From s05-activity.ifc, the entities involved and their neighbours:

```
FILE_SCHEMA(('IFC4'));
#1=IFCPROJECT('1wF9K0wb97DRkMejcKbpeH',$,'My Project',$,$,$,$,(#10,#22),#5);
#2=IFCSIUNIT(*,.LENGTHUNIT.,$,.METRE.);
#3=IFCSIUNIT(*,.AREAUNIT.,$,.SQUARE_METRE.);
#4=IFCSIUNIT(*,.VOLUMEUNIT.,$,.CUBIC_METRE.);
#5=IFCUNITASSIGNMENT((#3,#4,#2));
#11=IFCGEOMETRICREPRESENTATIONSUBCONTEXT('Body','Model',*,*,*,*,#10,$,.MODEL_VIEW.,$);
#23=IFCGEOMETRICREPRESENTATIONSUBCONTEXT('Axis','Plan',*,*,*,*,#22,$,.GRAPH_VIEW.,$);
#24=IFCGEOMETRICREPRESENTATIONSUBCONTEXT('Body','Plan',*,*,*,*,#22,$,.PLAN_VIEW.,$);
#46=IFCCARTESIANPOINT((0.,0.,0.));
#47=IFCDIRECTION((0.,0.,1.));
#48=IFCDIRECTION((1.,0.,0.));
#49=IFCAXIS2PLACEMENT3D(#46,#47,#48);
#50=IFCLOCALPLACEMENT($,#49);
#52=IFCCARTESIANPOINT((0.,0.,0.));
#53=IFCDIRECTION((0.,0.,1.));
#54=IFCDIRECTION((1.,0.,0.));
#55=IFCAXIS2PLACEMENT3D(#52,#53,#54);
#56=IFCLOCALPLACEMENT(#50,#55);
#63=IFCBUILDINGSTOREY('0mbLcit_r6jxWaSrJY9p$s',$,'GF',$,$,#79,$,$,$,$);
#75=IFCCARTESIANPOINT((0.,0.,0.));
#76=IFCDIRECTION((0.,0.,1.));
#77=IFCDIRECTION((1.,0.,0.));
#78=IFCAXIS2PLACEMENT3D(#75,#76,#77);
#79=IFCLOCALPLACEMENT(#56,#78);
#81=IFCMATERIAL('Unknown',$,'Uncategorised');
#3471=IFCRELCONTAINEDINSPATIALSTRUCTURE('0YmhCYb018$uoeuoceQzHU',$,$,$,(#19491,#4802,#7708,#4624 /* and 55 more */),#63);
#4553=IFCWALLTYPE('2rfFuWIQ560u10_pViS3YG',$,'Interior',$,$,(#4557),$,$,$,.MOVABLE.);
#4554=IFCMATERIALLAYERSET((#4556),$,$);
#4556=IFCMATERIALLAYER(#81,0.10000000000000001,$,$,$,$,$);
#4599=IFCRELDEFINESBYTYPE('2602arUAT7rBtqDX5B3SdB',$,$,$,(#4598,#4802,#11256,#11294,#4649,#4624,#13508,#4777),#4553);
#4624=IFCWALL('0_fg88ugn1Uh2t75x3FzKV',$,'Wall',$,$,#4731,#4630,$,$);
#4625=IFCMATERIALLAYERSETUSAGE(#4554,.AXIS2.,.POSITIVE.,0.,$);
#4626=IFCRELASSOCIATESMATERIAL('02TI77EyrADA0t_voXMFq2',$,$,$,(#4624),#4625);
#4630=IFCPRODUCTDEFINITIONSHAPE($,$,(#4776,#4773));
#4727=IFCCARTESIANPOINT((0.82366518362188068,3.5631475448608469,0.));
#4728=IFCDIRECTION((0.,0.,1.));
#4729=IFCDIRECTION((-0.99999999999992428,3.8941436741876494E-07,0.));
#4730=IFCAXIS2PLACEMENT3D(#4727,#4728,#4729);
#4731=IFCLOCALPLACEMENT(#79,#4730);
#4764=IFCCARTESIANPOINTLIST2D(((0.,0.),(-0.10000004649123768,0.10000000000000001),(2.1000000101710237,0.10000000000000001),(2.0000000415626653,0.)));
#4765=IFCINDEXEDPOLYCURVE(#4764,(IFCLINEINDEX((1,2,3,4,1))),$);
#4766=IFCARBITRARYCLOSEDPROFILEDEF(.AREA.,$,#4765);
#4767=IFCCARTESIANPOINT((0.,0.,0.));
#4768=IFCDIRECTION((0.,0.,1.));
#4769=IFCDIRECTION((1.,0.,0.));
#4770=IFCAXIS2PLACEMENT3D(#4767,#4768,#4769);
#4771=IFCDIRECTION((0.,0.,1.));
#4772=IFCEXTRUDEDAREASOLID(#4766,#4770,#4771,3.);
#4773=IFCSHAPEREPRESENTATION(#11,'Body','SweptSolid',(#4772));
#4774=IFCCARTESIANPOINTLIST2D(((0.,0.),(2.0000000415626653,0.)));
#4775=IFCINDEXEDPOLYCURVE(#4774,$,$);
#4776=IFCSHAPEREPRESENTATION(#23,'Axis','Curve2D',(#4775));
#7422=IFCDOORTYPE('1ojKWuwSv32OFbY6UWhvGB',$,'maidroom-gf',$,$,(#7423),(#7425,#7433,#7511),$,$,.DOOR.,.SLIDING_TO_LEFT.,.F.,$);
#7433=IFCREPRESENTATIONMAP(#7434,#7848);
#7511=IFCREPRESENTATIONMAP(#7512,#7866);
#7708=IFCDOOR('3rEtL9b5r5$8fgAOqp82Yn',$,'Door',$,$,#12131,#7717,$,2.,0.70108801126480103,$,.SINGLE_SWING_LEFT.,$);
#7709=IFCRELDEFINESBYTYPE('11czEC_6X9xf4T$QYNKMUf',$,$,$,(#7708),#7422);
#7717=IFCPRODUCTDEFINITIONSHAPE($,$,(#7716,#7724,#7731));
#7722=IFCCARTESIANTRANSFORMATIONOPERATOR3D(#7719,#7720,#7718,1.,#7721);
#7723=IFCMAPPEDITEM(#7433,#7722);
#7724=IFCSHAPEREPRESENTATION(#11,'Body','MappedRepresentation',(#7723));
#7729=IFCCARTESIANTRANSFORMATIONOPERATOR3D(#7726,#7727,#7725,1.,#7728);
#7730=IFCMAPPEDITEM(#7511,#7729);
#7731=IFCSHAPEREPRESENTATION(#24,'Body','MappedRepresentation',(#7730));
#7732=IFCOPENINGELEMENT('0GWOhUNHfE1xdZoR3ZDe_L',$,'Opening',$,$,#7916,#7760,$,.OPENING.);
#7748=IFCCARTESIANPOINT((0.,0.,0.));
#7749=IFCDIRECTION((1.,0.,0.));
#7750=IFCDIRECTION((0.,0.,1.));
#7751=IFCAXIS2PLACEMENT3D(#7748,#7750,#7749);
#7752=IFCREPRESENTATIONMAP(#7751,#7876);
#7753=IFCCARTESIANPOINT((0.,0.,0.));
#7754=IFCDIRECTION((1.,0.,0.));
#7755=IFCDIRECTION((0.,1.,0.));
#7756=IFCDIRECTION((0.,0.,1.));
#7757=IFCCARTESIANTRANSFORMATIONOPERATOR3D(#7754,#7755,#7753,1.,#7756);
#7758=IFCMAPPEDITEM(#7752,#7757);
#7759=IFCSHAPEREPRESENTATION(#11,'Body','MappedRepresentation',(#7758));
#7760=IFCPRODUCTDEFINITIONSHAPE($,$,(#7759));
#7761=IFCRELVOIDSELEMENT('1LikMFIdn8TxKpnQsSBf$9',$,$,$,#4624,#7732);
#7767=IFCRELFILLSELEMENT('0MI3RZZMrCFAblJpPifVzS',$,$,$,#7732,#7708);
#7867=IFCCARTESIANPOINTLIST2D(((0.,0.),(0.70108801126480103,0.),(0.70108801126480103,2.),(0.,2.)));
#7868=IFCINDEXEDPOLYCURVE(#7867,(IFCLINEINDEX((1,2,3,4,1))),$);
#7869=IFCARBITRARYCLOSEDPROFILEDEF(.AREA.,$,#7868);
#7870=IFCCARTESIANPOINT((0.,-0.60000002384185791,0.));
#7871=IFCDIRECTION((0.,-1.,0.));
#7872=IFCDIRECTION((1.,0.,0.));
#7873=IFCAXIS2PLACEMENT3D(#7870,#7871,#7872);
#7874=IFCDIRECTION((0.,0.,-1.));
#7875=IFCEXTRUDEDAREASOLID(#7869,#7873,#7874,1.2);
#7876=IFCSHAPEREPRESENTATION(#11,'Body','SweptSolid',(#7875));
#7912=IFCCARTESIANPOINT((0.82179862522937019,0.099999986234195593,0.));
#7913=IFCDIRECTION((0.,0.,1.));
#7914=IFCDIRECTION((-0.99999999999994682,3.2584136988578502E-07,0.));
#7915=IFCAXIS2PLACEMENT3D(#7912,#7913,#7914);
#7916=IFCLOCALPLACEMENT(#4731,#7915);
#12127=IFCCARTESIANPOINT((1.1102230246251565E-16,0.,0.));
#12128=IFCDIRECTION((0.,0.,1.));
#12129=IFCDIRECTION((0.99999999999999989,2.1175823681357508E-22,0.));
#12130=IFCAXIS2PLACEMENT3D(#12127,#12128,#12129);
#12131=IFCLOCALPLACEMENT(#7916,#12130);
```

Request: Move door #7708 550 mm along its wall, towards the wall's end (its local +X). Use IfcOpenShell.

```python
import ifcopenshell
import ifcopenshell.api.geometry
import ifcopenshell.util.placement
import ifcopenshell.util.unit

model = ifcopenshell.open("s05-activity.ifc")
unit_scale = ifcopenshell.util.unit.calculate_unit_scale(model)

door = model.by_id(7708)
opening = door.FillsVoids[0].RelatingOpeningElement
wall = opening.VoidsElements[0].RelatingBuildingElement

wall_matrix = ifcopenshell.util.placement.get_local_placement(wall.ObjectPlacement)
shift = wall_matrix[:3, 0] * 0.55 / unit_scale
before = ifcopenshell.util.placement.get_local_placement(door.ObjectPlacement)[:3, 3].copy()

# The door is placed relative to its opening, so it follows when the opening moves.
matrix = ifcopenshell.util.placement.get_local_placement(opening.ObjectPlacement)
matrix[:3, 3] += shift
ifcopenshell.api.geometry.edit_object_placement(
    model, product=opening, matrix=matrix, is_si=False, should_transform_children=True
)

after = ifcopenshell.util.placement.get_local_placement(door.ObjectPlacement)[:3, 3]
print("door moved by", (after - before).round(3) + 0.0)

model.write("s05-activity_updated.ifc")
```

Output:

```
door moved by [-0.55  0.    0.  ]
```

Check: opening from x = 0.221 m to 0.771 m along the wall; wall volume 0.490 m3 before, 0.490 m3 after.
